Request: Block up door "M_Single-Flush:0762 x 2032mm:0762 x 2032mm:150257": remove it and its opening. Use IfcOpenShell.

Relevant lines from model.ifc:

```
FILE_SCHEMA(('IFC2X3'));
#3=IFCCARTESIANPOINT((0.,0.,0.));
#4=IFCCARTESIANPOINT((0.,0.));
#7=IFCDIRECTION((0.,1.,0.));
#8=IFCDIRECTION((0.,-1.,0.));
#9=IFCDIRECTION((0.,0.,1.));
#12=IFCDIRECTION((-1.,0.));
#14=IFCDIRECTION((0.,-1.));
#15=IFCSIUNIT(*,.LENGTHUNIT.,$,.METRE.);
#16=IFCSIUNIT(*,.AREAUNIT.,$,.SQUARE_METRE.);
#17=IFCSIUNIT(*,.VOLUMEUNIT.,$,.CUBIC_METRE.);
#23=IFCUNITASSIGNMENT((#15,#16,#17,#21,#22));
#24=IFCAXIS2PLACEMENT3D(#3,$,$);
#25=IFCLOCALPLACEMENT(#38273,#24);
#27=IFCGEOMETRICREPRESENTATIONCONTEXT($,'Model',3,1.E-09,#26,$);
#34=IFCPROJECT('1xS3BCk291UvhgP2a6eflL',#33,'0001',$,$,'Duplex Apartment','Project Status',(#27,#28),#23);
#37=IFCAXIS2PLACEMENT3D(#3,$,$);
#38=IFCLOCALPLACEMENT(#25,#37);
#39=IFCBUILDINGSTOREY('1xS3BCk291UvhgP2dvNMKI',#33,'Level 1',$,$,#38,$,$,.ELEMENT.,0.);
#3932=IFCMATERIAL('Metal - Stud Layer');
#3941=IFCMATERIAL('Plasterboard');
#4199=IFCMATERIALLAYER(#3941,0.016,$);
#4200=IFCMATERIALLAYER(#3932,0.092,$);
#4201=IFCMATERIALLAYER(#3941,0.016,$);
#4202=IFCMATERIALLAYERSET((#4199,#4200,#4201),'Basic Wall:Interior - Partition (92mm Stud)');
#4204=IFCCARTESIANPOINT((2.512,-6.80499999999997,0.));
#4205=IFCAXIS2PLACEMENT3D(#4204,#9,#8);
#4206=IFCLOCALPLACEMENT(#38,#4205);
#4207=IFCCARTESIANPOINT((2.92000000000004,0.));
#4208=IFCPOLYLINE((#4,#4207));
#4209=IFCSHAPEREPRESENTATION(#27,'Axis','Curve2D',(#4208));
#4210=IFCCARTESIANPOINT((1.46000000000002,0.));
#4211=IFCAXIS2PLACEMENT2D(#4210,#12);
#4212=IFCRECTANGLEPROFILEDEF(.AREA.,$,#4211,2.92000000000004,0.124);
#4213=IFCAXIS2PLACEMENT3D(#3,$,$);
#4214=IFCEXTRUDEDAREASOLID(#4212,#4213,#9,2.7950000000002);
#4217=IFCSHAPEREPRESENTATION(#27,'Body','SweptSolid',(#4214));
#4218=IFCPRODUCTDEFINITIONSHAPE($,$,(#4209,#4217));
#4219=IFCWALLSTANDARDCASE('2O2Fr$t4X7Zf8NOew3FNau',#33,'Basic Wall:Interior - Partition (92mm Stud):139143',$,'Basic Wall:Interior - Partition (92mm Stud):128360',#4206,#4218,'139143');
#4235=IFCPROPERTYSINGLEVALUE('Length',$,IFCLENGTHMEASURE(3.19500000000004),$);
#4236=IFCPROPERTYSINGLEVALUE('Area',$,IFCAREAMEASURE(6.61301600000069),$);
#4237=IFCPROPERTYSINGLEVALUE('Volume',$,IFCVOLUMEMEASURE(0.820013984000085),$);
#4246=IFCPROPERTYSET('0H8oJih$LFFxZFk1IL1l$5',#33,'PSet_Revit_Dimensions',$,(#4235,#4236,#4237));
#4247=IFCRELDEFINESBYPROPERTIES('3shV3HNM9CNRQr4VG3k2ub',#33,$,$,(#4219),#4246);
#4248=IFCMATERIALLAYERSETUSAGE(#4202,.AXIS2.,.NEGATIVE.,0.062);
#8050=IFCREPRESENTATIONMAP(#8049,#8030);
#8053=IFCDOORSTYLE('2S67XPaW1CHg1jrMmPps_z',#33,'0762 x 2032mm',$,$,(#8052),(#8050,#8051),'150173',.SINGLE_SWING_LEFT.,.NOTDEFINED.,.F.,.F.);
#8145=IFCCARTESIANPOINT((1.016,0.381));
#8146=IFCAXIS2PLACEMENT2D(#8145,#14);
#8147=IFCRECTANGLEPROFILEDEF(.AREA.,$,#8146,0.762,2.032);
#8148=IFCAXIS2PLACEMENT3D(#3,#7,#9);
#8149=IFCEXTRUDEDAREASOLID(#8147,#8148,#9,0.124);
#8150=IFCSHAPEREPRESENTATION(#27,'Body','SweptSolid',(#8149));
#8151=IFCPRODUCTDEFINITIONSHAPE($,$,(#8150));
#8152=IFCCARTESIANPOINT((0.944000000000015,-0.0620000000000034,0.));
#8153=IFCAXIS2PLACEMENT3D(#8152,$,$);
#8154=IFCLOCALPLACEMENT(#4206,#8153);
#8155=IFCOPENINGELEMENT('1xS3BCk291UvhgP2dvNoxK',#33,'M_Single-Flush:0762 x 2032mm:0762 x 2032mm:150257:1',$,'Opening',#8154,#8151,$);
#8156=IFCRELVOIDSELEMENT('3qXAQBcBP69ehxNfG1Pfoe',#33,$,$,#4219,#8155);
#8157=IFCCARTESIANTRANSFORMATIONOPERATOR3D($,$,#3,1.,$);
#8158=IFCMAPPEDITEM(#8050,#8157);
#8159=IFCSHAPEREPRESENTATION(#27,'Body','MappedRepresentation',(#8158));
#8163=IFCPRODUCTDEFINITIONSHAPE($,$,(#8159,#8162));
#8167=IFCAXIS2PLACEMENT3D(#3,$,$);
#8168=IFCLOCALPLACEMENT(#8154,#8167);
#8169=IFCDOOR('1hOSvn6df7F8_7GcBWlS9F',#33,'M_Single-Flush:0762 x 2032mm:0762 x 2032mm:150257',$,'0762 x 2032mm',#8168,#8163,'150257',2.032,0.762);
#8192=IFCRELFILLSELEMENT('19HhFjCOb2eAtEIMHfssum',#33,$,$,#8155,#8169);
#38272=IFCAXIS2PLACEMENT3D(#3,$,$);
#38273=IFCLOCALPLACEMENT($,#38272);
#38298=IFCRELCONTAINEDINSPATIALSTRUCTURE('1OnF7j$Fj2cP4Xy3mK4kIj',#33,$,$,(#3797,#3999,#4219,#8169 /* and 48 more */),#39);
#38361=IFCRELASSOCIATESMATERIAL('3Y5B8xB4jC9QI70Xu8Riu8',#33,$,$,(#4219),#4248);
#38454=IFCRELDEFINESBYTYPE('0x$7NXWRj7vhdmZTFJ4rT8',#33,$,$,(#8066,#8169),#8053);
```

```python
import ifcopenshell
import ifcopenshell.api.feature
import ifcopenshell.api.pset
import ifcopenshell.api.root
import ifcopenshell.geom
import ifcopenshell.util.element
import ifcopenshell.util.shape
import ifcopenshell.util.unit

model = ifcopenshell.open("model.ifc")
area_scale = ifcopenshell.util.unit.calculate_unit_scale(model, "AREAUNIT")
volume_scale = ifcopenshell.util.unit.calculate_unit_scale(model, "VOLUMEUNIT")
settings = ifcopenshell.geom.settings()


def volume(element):
    """Net volume in cubic metres, openings subtracted."""
    shape = ifcopenshell.geom.create_shape(settings, element)
    return ifcopenshell.util.shape.get_volume(shape.geometry)


door = model.by_id(8169)
opening = door.FillsVoids[0].RelatingOpeningElement
wall = opening.VoidsElements[0].RelatingBuildingElement
before = volume(wall)

ifcopenshell.api.root.remove_product(model, product=door)
ifcopenshell.api.feature.remove_feature(model, feature=opening)

after = volume(wall)
thickness = 0.124  # wall thickness in metres

# Update the wall's stored quantities.
pset = model.by_id(ifcopenshell.util.element.get_pset(wall, "PSet_Revit_Dimensions", should_inherit=False)["id"])
ifcopenshell.api.pset.edit_pset(model, pset=pset, properties={
    "Area": model.create_entity("IfcAreaMeasure", after / thickness / area_scale),
    "Volume": model.create_entity("IfcVolumeMeasure", after / volume_scale),
})

print(f"wall volume {before:.3f} -> {after:.3f} m3")

model.write("model_v2.ifc")
```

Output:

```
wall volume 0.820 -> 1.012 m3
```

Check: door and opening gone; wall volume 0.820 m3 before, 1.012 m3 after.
